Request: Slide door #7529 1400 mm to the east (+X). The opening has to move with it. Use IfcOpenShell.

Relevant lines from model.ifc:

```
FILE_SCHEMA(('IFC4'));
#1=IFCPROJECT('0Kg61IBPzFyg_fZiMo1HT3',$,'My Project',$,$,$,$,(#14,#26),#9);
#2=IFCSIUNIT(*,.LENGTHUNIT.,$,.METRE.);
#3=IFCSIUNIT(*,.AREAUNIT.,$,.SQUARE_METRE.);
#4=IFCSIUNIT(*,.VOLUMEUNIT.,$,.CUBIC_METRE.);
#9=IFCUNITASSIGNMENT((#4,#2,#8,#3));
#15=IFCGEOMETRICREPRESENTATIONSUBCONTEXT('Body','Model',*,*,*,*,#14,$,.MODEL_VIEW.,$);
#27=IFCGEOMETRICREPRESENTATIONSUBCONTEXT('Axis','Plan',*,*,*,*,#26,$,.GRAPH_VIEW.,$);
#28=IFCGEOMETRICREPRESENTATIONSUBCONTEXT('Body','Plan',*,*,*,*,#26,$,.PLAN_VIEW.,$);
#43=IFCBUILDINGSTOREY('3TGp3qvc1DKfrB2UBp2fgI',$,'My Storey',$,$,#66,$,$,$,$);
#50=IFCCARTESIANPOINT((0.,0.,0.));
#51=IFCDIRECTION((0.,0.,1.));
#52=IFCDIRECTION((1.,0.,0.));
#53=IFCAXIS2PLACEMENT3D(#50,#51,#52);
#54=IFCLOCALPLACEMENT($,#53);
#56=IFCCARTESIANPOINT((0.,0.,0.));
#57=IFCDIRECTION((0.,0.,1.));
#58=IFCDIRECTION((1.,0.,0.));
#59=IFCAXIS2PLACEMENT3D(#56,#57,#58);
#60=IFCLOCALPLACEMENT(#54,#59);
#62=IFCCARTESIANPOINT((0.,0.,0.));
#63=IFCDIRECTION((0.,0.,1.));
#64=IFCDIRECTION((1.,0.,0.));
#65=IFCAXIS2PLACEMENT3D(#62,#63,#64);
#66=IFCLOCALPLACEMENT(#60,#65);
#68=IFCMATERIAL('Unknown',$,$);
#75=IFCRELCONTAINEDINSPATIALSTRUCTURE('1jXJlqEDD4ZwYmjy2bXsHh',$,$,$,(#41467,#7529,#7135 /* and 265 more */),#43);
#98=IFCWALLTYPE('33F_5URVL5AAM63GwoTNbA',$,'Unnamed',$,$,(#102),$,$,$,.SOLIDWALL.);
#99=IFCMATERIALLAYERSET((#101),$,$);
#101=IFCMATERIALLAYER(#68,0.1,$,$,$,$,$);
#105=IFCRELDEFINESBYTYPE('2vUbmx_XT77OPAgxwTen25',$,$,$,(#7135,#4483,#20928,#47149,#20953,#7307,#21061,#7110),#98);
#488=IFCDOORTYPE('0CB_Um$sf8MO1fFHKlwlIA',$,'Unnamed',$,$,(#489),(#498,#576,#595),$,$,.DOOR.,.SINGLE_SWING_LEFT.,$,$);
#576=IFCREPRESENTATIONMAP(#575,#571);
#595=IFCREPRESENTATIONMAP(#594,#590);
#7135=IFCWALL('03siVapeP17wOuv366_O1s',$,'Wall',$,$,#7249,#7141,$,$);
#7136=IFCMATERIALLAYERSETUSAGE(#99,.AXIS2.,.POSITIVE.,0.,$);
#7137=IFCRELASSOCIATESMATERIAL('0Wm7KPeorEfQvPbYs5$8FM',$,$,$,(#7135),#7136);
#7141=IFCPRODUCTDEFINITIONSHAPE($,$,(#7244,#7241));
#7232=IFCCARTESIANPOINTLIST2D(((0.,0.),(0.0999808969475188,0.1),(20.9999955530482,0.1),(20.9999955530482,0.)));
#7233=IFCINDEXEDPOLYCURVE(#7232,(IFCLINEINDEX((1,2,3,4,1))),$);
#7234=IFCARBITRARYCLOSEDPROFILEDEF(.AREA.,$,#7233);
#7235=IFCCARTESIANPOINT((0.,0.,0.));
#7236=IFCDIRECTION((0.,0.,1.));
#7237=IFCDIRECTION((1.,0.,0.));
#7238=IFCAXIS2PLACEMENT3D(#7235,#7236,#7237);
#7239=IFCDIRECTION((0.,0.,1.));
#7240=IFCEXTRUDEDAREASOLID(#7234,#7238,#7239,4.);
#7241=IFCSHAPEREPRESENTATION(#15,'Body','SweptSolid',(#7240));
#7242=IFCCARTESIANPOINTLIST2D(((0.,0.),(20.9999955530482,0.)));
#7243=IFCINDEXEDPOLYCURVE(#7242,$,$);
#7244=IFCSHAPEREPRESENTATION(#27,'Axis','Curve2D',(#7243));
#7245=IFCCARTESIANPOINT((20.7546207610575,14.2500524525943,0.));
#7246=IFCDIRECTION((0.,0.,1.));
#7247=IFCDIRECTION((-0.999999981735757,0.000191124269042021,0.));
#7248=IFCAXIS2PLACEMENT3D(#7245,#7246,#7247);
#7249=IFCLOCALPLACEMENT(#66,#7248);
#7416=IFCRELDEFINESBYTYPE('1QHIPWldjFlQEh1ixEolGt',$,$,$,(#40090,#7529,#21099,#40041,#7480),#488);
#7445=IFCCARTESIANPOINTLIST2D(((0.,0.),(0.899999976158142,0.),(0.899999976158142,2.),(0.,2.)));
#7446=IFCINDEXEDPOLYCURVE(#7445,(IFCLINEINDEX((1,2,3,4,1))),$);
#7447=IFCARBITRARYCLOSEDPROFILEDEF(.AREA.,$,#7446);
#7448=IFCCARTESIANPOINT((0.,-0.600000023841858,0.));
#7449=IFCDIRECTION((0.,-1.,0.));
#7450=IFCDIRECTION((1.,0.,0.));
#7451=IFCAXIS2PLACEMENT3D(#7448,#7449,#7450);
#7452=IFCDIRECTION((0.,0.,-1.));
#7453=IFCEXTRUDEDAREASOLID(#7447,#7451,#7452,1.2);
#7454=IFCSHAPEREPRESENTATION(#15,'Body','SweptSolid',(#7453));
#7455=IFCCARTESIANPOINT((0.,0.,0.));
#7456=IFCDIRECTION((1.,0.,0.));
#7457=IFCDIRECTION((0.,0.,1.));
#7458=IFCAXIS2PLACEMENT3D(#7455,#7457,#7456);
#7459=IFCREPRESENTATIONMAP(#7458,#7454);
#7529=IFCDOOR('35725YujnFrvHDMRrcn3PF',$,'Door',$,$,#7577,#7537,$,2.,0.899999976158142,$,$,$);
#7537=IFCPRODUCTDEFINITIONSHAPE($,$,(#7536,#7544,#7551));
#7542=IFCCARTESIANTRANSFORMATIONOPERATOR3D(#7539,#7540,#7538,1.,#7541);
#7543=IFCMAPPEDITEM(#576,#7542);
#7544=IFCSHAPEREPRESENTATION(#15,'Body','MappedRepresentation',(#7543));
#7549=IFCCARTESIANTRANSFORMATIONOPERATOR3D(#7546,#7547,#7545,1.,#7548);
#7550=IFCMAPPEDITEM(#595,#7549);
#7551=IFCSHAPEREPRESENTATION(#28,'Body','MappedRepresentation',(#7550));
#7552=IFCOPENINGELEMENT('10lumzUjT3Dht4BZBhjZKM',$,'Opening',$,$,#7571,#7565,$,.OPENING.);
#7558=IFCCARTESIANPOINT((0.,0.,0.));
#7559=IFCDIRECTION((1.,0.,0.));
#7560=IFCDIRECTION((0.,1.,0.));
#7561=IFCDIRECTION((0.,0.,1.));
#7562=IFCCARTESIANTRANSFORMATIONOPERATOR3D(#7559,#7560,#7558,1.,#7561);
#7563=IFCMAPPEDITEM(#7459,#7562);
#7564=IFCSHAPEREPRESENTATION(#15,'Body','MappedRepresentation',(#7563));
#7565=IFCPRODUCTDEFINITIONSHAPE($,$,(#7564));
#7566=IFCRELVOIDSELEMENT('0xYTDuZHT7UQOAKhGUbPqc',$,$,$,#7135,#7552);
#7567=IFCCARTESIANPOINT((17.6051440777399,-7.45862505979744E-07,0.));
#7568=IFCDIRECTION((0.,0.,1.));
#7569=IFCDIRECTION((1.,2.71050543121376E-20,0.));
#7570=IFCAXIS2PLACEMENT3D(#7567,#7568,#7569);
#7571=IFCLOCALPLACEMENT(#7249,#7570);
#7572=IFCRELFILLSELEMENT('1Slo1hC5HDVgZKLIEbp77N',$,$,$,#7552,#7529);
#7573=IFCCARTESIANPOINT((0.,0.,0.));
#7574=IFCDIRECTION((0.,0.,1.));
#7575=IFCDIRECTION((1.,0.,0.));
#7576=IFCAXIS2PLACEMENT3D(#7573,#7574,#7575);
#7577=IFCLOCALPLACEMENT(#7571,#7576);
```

```python
import ifcopenshell
import ifcopenshell.api.geometry
import ifcopenshell.util.placement
import ifcopenshell.util.unit

model = ifcopenshell.open("model.ifc")
unit_scale = ifcopenshell.util.unit.calculate_unit_scale(model)

door = model.by_guid("35725YujnFrvHDMRrcn3PF")
opening = door.FillsVoids[0].RelatingOpeningElement
wall = opening.VoidsElements[0].RelatingBuildingElement

wall_matrix = ifcopenshell.util.placement.get_local_placement(wall.ObjectPlacement)
shift = wall_matrix[:3, 0] * -1.4 / unit_scale
before = ifcopenshell.util.placement.get_local_placement(door.ObjectPlacement)[:3, 3].copy()

# The door is placed relative to its opening, so it follows when the opening moves.
matrix = ifcopenshell.util.placement.get_local_placement(opening.ObjectPlacement)
matrix[:3, 3] += shift
ifcopenshell.api.geometry.edit_object_placement(
    model, product=opening, matrix=matrix, is_si=False, should_transform_children=True
)

after = ifcopenshell.util.placement.get_local_placement(door.ObjectPlacement)[:3, 3]
print("door moved by", (after - before).round(3) + 0.0)

model.write("model-out.ifc")
```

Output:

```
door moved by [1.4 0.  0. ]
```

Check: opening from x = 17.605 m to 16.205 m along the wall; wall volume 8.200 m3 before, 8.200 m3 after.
